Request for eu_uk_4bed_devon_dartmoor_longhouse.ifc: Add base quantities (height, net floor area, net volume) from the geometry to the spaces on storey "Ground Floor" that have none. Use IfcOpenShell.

First a look at what the model holds.

```python
import ifcopenshell
import ifcopenshell.util.element
import ifcopenshell.util.unit

model = ifcopenshell.open("eu_uk_4bed_devon_dartmoor_longhouse.ifc")
print(model.schema)
for unit_type in ("LENGTHUNIT", "AREAUNIT", "VOLUMEUNIT"):
    print(unit_type, ifcopenshell.util.unit.calculate_unit_scale(model, unit_type))
storey = next(s for s in model.by_type("IfcBuildingStorey") if s.Name == "Ground Floor")
spaces = [e for e in ifcopenshell.util.element.get_decomposition(storey) if e.is_a("IfcSpace")]
for e in sorted(spaces, key=lambda e: e.id()):
    print(e.id(), e.is_a(), e.Name, list(ifcopenshell.util.element.get_psets(e, qtos_only=True)), sep=" | ")
```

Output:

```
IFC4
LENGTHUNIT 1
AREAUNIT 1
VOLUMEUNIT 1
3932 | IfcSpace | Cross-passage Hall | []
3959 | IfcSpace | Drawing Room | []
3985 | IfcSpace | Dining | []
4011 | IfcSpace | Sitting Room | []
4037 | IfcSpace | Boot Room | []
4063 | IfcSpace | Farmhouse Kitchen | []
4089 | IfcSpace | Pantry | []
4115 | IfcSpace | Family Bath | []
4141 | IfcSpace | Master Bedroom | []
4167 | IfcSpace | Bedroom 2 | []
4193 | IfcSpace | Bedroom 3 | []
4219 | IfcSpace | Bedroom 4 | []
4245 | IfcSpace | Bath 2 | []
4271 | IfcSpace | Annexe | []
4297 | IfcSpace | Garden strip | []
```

```python
import ifcopenshell
import ifcopenshell.api.pset
import ifcopenshell.geom
import ifcopenshell.util.element
import ifcopenshell.util.shape
import ifcopenshell.util.unit

model = ifcopenshell.open("eu_uk_4bed_devon_dartmoor_longhouse.ifc")
unit_scale = ifcopenshell.util.unit.calculate_unit_scale(model)
area_scale = ifcopenshell.util.unit.calculate_unit_scale(model, "AREAUNIT")
volume_scale = ifcopenshell.util.unit.calculate_unit_scale(model, "VOLUMEUNIT")
settings = ifcopenshell.geom.settings()

storey = next(s for s in model.by_type("IfcBuildingStorey") if s.Name == "Ground Floor")
spaces = [e for e in ifcopenshell.util.element.get_decomposition(storey) if e.is_a("IfcSpace")]

for e in sorted(spaces, key=lambda e: e.id()):
    if ifcopenshell.util.element.get_psets(e, qtos_only=True, should_inherit=False):
        continue
    # Geometry comes back in metres, in the element's own axes.
    shape = ifcopenshell.geom.create_shape(settings, e)
    values = {
        "Height": ifcopenshell.util.shape.get_z(shape.geometry) / unit_scale,
        "NetFloorArea": ifcopenshell.util.shape.get_footprint_area(shape.geometry) / area_scale,
        "NetVolume": ifcopenshell.util.shape.get_volume(shape.geometry) / volume_scale,
    }
    qto = ifcopenshell.api.pset.add_qto(model, product=e, name="Qto_SpaceBaseQuantities")
    ifcopenshell.api.pset.edit_qto(model, qto=qto, properties=values)
    print(e.id(), {k: round(v, 3) for k, v in values.items()})

model.write("eu_uk_4bed_devon_dartmoor_longhouse_updated.ifc")
```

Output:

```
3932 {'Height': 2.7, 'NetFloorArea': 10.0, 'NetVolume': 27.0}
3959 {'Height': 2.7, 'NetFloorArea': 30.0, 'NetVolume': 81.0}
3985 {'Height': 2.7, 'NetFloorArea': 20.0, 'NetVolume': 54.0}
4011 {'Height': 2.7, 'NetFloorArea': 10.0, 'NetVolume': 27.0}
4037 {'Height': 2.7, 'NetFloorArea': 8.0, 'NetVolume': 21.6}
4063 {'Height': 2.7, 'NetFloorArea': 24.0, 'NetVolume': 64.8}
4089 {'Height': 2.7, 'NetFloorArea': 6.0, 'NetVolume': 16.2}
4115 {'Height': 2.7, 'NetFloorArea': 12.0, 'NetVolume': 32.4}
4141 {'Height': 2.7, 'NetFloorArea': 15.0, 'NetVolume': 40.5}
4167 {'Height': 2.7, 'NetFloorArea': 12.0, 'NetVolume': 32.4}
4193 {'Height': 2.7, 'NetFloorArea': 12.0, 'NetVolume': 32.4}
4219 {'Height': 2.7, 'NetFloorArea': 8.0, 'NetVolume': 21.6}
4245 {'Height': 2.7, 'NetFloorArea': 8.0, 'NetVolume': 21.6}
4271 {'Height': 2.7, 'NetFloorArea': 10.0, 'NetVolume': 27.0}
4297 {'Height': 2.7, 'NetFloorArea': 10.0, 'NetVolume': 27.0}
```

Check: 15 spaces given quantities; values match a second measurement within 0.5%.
